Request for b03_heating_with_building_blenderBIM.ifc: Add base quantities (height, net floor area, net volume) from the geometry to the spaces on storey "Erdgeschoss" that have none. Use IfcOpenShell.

First a look at what the model holds.

```python
import ifcopenshell
import ifcopenshell.util.element
import ifcopenshell.util.unit

model = ifcopenshell.open("b03_heating_with_building_blenderBIM.ifc")
print(model.schema)
for unit_type in ("LENGTHUNIT", "AREAUNIT", "VOLUMEUNIT"):
    print(unit_type, ifcopenshell.util.unit.calculate_unit_scale(model, unit_type))
storey = next(s for s in model.by_type("IfcBuildingStorey") if s.Name == "Erdgeschoss")
spaces = [e for e in ifcopenshell.util.element.get_decomposition(storey) if e.is_a("IfcSpace")]
for e in sorted(spaces, key=lambda e: e.id()):
    print(e.id(), e.is_a(), e.Name, list(ifcopenshell.util.element.get_psets(e, qtos_only=True)), sep=" | ")
```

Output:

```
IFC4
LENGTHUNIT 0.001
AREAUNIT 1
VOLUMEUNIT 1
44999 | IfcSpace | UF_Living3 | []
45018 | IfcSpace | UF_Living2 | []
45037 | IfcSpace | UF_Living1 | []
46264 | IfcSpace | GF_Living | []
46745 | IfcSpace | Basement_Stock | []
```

```python
import ifcopenshell
import ifcopenshell.api.pset
import ifcopenshell.geom
import ifcopenshell.util.element
import ifcopenshell.util.shape
import ifcopenshell.util.unit

model = ifcopenshell.open("b03_heating_with_building_blenderBIM.ifc")
unit_scale = ifcopenshell.util.unit.calculate_unit_scale(model)
area_scale = ifcopenshell.util.unit.calculate_unit_scale(model, "AREAUNIT")
volume_scale = ifcopenshell.util.unit.calculate_unit_scale(model, "VOLUMEUNIT")
settings = ifcopenshell.geom.settings()

storey = next(s for s in model.by_type("IfcBuildingStorey") if s.Name == "Erdgeschoss")
spaces = [e for e in ifcopenshell.util.element.get_decomposition(storey) if e.is_a("IfcSpace")]

for e in sorted(spaces, key=lambda e: e.id()):
    if ifcopenshell.util.element.get_psets(e, qtos_only=True, should_inherit=False):
        continue
    # Geometry comes back in metres, in the element's own axes.
    shape = ifcopenshell.geom.create_shape(settings, e)
    values = {
        "Height": ifcopenshell.util.shape.get_z(shape.geometry) / unit_scale,
        "NetFloorArea": ifcopenshell.util.shape.get_footprint_area(shape.geometry) / area_scale,
        "NetVolume": ifcopenshell.util.shape.get_volume(shape.geometry) / volume_scale,
    }
    qto = ifcopenshell.api.pset.add_qto(model, product=e, name="Qto_SpaceBaseQuantities")
    ifcopenshell.api.pset.edit_qto(model, qto=qto, properties=values)
    print(e.id(), {k: round(v, 3) for k, v in values.items()})

model.write("b03_heating_with_building_blenderBIM_rev.ifc")
```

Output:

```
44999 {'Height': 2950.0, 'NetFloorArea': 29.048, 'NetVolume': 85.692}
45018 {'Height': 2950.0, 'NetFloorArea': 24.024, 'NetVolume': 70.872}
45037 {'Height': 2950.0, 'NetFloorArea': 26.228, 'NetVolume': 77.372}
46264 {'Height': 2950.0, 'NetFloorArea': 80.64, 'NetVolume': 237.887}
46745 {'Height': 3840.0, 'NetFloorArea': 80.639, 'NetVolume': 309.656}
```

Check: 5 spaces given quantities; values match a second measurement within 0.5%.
